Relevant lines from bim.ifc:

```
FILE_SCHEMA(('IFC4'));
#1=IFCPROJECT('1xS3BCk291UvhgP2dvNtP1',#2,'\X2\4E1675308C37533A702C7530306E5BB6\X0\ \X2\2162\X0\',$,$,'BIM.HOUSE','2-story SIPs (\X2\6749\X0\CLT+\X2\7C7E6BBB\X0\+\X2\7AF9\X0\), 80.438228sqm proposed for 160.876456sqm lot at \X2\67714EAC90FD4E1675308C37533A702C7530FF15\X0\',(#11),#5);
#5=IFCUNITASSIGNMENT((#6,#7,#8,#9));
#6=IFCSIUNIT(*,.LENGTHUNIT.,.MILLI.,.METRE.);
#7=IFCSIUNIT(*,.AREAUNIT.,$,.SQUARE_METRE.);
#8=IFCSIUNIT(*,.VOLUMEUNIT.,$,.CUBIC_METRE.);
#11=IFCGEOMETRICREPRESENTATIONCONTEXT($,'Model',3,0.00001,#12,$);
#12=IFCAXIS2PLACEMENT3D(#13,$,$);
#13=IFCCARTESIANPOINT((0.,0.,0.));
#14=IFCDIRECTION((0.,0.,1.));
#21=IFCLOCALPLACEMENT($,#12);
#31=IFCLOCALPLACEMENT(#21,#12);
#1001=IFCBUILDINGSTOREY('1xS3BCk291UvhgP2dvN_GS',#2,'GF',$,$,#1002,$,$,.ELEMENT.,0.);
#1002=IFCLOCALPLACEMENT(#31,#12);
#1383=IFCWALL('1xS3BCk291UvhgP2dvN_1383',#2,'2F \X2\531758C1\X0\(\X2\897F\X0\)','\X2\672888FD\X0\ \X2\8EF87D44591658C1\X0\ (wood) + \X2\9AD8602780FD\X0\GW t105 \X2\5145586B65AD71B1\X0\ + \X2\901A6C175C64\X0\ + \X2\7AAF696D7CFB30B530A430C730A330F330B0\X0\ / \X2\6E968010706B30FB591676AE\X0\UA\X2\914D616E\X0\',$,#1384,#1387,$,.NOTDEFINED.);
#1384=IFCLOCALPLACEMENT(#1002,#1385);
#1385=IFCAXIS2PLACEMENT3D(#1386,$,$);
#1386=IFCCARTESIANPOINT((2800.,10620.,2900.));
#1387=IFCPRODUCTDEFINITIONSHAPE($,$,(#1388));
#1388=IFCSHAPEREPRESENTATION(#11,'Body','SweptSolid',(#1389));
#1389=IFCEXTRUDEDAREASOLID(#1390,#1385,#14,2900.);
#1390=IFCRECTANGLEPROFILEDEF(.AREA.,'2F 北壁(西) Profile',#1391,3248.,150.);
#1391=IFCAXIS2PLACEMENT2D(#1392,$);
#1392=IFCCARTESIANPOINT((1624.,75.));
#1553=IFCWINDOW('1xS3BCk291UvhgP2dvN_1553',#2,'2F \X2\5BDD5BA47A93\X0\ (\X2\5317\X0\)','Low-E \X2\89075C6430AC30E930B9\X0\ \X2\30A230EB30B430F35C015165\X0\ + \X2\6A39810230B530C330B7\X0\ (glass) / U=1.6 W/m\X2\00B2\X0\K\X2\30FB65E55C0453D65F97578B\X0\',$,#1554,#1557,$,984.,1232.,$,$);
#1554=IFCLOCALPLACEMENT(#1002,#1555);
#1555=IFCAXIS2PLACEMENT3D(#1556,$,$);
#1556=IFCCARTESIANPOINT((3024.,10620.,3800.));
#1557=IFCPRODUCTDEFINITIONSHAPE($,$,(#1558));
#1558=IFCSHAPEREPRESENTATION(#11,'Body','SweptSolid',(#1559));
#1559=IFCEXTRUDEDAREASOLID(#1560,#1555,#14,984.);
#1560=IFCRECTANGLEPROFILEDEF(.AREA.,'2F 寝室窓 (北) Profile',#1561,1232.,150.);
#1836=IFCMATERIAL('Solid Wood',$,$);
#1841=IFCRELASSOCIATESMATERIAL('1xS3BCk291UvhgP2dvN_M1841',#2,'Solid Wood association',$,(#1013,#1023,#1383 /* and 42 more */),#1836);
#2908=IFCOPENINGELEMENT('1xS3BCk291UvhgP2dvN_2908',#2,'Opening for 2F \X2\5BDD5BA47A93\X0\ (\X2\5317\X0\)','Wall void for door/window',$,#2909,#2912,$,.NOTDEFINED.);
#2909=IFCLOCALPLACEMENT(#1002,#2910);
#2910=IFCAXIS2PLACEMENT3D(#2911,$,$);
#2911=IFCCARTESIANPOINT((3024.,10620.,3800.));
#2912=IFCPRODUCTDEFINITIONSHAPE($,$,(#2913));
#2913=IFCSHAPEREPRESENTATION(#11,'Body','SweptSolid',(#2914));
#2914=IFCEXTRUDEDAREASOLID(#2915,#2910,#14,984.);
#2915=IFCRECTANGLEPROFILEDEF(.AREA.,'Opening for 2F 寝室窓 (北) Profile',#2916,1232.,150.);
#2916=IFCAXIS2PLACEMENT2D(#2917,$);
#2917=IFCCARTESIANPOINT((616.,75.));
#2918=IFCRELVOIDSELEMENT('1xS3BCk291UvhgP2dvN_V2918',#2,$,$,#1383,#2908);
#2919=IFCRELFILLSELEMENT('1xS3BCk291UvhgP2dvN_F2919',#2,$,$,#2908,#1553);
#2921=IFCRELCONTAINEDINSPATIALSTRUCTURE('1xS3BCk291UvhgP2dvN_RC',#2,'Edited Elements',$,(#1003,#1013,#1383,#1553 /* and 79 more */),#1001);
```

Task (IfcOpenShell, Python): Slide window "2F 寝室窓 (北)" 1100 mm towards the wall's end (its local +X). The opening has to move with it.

```python
import ifcopenshell
import ifcopenshell.api.geometry
import ifcopenshell.util.placement

model = ifcopenshell.open("bim.ifc")

window = model.by_guid("1xS3BCk291UvhgP2dvN_1553")
opening = window.FillsVoids[0].RelatingOpeningElement
wall = opening.VoidsElements[0].RelatingBuildingElement

wall_matrix = ifcopenshell.util.placement.get_local_placement(wall.ObjectPlacement)
shift = wall_matrix[:3, 0] * 1100.0
before = ifcopenshell.util.placement.get_local_placement(window.ObjectPlacement)[:3, 3].copy()

# The window is not placed relative to its opening, so move both.
for product in (opening, window):
    matrix = ifcopenshell.util.placement.get_local_placement(product.ObjectPlacement)
    matrix[:3, 3] += shift
    ifcopenshell.api.geometry.edit_object_placement(model, product=product, matrix=matrix, is_si=False)

after = ifcopenshell.util.placement.get_local_placement(window.ObjectPlacement)[:3, 3]
print("window moved by", (after - before).round(3) + 0.0)

model.write("bim_v2.ifc")
```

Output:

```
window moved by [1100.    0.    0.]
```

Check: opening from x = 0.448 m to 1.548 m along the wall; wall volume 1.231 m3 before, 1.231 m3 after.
